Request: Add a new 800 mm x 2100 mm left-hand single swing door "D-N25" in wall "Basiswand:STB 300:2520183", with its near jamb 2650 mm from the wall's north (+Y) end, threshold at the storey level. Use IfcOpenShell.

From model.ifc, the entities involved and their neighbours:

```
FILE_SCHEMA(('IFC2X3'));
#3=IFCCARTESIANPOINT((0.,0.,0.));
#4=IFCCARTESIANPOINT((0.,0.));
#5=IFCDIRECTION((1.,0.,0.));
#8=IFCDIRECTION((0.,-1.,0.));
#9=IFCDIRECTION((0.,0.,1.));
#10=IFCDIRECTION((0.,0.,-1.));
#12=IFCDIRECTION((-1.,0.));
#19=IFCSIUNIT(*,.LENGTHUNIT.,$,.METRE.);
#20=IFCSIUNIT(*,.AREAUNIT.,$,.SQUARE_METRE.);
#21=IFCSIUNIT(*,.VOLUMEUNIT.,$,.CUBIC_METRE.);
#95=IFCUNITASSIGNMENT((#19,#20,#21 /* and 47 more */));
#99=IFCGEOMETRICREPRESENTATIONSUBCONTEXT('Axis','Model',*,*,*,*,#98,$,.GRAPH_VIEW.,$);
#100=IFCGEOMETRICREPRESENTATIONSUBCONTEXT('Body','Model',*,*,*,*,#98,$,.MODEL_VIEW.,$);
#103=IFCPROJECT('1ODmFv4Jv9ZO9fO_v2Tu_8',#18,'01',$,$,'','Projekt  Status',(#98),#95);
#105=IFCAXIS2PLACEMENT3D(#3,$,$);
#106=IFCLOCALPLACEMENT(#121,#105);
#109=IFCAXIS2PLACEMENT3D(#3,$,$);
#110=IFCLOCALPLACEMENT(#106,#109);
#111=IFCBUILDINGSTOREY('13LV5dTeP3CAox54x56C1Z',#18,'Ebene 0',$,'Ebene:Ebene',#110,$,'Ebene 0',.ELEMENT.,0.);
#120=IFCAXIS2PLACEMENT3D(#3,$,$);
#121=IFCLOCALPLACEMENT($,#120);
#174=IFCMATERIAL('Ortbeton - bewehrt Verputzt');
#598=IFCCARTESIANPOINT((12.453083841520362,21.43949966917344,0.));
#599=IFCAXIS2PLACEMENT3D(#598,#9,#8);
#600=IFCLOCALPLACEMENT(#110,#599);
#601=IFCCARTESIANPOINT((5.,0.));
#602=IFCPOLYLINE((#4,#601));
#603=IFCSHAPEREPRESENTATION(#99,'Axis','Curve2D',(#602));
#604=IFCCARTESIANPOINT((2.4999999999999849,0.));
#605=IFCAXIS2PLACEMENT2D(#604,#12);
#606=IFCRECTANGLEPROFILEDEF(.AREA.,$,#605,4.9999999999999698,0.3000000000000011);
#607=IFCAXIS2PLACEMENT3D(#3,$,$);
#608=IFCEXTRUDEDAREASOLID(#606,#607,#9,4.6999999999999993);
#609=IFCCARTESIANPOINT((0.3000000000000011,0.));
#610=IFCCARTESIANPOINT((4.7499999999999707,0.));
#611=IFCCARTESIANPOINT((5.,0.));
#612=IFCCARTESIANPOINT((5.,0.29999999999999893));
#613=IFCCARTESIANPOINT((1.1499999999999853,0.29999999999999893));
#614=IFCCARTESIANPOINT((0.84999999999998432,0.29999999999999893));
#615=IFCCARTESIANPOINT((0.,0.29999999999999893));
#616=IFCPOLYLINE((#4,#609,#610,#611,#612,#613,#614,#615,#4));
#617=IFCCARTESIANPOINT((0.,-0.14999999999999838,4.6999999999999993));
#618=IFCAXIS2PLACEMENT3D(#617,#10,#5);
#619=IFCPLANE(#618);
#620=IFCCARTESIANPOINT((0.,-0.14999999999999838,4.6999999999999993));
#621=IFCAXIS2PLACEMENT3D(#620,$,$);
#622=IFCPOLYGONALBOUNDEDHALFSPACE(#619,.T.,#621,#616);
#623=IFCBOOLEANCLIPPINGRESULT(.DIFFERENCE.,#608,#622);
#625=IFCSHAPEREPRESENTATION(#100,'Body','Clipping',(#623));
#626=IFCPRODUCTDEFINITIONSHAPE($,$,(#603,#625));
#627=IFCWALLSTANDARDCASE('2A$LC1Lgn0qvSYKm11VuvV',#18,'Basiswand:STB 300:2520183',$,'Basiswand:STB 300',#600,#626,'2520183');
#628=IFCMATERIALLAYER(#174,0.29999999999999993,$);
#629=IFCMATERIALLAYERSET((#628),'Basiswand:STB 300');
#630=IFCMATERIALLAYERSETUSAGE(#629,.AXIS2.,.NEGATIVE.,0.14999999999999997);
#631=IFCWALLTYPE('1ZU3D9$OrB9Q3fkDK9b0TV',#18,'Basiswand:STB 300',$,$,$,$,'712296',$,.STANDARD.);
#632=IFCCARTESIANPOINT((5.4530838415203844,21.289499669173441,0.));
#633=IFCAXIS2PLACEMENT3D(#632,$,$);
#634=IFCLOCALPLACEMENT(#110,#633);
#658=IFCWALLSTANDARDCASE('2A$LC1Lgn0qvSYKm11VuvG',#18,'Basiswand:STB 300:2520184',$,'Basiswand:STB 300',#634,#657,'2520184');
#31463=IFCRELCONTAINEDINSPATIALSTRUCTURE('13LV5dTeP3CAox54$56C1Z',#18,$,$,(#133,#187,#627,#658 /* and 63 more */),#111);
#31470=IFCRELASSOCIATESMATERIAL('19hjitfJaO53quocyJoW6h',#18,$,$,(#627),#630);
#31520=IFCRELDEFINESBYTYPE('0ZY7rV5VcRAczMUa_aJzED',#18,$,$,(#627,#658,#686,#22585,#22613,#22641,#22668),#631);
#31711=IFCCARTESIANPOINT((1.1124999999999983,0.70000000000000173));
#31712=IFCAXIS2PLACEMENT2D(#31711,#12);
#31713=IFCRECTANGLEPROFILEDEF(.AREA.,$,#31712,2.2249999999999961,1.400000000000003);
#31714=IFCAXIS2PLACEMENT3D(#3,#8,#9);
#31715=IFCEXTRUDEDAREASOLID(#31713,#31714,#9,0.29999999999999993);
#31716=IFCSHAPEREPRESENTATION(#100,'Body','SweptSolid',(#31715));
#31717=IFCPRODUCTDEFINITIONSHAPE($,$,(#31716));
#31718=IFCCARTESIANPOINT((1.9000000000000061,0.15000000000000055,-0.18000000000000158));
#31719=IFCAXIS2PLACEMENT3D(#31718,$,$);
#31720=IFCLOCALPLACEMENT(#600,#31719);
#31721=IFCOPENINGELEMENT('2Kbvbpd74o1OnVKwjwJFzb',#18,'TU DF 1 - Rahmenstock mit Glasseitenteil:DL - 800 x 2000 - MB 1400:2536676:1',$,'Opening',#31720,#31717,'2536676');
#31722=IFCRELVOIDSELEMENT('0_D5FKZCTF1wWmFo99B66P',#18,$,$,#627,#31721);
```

```python
import numpy as np
import ifcopenshell
import ifcopenshell.api.feature
import ifcopenshell.api.geometry
import ifcopenshell.api.root
import ifcopenshell.api.spatial
import ifcopenshell.api.type
import ifcopenshell.geom
import ifcopenshell.util.element
import ifcopenshell.util.placement
import ifcopenshell.util.representation
import ifcopenshell.util.shape
import ifcopenshell.util.unit

model = ifcopenshell.open("model.ifc")
unit_scale = ifcopenshell.util.unit.calculate_unit_scale(model)
settings = ifcopenshell.geom.settings()


def volume(element):
    """Net volume in cubic metres, openings subtracted."""
    shape = ifcopenshell.geom.create_shape(settings, element)
    return ifcopenshell.util.shape.get_volume(shape.geometry)


wall = model.by_id(627)
storey = ifcopenshell.util.element.get_container(wall, ifc_class="IfcBuildingStorey")
context = ifcopenshell.util.representation.get_context(model, "Model", "Body", "MODEL_VIEW")
before = volume(wall)

width, height, from_end, sill = 0.8, 2.1, 2.65, 0.0  # metres

# The wall runs along its own X axis, and the end named is its -X end.
wall_shape = ifcopenshell.geom.create_shape(settings, wall)
x, y, z = ifcopenshell.util.shape.get_vertices(wall_shape.geometry).T
start = x.min() + from_end
face, thickness = float(y.min()), float(y.max() - y.min())
wall_matrix = ifcopenshell.util.placement.get_local_placement(wall.ObjectPlacement)
level = ifcopenshell.util.placement.get_local_placement(storey.ObjectPlacement)[2, 3]


def in_wall(x, y):
    """Placement at x, y metres in the wall's axes, at sill height."""
    matrix = wall_matrix.copy()
    matrix[:, 3] = wall_matrix @ np.array([x / unit_scale, y / unit_scale, 0.0, 1.0])
    matrix[2, 3] = level + sill / unit_scale
    return matrix


# Opening: a box that overshoots both wall faces by 50 mm.
opening = ifcopenshell.api.root.create_entity(model, ifc_class="IfcOpeningElement")
box = ifcopenshell.api.geometry.add_wall_representation(
    model, context=context, length=width, height=height, thickness=thickness + 0.1
)
ifcopenshell.api.geometry.assign_representation(model, product=opening, representation=box)
ifcopenshell.api.geometry.edit_object_placement(model, product=opening, matrix=in_wall(start, face - 0.05), is_si=False)
ifcopenshell.api.feature.add_feature(model, feature=opening, element=wall)

door = ifcopenshell.api.root.create_entity(model, ifc_class="IfcDoor", name="D-N25")
door.OverallWidth, door.OverallHeight = width / unit_scale, height / unit_scale
body = ifcopenshell.api.geometry.add_door_representation(
    model,
    context=context,
    overall_width=door.OverallWidth,
    overall_height=door.OverallHeight,
    operation_type="SINGLE_SWING_LEFT",
    lining_properties={"LiningDepth": thickness / unit_scale, "ThresholdDepth": thickness / unit_scale},
)
ifcopenshell.api.geometry.assign_representation(model, product=door, representation=body)
ifcopenshell.api.spatial.assign_container(model, products=[door], relating_structure=storey)
fills = ifcopenshell.api.feature.add_filling(model, opening=opening, element=door)
fills.OwnerHistory = door.OwnerHistory  # required in IFC2X3

# IFC2X3 keeps the operation on the door style.
style = ifcopenshell.api.root.create_entity(model, ifc_class="IfcDoorStyle", name="D-N25")
style.OperationType, style.ConstructionType = "SINGLE_SWING_LEFT", "NOTDEFINED"
style.ParameterTakesPrecedence = style.Sizeable = False
ifcopenshell.api.type.assign_type(model, related_objects=[door], relating_type=style)

# The lining spans the wall, so the door starts at the wall face.
ifcopenshell.api.geometry.edit_object_placement(model, product=door, matrix=in_wall(start, face), is_si=False)

after = volume(wall)

print(f"wall volume {before:.3f} -> {after:.3f} m3")

model.write("model_updated.ifc")
```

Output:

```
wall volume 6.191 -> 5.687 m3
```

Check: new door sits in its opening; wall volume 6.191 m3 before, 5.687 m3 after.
